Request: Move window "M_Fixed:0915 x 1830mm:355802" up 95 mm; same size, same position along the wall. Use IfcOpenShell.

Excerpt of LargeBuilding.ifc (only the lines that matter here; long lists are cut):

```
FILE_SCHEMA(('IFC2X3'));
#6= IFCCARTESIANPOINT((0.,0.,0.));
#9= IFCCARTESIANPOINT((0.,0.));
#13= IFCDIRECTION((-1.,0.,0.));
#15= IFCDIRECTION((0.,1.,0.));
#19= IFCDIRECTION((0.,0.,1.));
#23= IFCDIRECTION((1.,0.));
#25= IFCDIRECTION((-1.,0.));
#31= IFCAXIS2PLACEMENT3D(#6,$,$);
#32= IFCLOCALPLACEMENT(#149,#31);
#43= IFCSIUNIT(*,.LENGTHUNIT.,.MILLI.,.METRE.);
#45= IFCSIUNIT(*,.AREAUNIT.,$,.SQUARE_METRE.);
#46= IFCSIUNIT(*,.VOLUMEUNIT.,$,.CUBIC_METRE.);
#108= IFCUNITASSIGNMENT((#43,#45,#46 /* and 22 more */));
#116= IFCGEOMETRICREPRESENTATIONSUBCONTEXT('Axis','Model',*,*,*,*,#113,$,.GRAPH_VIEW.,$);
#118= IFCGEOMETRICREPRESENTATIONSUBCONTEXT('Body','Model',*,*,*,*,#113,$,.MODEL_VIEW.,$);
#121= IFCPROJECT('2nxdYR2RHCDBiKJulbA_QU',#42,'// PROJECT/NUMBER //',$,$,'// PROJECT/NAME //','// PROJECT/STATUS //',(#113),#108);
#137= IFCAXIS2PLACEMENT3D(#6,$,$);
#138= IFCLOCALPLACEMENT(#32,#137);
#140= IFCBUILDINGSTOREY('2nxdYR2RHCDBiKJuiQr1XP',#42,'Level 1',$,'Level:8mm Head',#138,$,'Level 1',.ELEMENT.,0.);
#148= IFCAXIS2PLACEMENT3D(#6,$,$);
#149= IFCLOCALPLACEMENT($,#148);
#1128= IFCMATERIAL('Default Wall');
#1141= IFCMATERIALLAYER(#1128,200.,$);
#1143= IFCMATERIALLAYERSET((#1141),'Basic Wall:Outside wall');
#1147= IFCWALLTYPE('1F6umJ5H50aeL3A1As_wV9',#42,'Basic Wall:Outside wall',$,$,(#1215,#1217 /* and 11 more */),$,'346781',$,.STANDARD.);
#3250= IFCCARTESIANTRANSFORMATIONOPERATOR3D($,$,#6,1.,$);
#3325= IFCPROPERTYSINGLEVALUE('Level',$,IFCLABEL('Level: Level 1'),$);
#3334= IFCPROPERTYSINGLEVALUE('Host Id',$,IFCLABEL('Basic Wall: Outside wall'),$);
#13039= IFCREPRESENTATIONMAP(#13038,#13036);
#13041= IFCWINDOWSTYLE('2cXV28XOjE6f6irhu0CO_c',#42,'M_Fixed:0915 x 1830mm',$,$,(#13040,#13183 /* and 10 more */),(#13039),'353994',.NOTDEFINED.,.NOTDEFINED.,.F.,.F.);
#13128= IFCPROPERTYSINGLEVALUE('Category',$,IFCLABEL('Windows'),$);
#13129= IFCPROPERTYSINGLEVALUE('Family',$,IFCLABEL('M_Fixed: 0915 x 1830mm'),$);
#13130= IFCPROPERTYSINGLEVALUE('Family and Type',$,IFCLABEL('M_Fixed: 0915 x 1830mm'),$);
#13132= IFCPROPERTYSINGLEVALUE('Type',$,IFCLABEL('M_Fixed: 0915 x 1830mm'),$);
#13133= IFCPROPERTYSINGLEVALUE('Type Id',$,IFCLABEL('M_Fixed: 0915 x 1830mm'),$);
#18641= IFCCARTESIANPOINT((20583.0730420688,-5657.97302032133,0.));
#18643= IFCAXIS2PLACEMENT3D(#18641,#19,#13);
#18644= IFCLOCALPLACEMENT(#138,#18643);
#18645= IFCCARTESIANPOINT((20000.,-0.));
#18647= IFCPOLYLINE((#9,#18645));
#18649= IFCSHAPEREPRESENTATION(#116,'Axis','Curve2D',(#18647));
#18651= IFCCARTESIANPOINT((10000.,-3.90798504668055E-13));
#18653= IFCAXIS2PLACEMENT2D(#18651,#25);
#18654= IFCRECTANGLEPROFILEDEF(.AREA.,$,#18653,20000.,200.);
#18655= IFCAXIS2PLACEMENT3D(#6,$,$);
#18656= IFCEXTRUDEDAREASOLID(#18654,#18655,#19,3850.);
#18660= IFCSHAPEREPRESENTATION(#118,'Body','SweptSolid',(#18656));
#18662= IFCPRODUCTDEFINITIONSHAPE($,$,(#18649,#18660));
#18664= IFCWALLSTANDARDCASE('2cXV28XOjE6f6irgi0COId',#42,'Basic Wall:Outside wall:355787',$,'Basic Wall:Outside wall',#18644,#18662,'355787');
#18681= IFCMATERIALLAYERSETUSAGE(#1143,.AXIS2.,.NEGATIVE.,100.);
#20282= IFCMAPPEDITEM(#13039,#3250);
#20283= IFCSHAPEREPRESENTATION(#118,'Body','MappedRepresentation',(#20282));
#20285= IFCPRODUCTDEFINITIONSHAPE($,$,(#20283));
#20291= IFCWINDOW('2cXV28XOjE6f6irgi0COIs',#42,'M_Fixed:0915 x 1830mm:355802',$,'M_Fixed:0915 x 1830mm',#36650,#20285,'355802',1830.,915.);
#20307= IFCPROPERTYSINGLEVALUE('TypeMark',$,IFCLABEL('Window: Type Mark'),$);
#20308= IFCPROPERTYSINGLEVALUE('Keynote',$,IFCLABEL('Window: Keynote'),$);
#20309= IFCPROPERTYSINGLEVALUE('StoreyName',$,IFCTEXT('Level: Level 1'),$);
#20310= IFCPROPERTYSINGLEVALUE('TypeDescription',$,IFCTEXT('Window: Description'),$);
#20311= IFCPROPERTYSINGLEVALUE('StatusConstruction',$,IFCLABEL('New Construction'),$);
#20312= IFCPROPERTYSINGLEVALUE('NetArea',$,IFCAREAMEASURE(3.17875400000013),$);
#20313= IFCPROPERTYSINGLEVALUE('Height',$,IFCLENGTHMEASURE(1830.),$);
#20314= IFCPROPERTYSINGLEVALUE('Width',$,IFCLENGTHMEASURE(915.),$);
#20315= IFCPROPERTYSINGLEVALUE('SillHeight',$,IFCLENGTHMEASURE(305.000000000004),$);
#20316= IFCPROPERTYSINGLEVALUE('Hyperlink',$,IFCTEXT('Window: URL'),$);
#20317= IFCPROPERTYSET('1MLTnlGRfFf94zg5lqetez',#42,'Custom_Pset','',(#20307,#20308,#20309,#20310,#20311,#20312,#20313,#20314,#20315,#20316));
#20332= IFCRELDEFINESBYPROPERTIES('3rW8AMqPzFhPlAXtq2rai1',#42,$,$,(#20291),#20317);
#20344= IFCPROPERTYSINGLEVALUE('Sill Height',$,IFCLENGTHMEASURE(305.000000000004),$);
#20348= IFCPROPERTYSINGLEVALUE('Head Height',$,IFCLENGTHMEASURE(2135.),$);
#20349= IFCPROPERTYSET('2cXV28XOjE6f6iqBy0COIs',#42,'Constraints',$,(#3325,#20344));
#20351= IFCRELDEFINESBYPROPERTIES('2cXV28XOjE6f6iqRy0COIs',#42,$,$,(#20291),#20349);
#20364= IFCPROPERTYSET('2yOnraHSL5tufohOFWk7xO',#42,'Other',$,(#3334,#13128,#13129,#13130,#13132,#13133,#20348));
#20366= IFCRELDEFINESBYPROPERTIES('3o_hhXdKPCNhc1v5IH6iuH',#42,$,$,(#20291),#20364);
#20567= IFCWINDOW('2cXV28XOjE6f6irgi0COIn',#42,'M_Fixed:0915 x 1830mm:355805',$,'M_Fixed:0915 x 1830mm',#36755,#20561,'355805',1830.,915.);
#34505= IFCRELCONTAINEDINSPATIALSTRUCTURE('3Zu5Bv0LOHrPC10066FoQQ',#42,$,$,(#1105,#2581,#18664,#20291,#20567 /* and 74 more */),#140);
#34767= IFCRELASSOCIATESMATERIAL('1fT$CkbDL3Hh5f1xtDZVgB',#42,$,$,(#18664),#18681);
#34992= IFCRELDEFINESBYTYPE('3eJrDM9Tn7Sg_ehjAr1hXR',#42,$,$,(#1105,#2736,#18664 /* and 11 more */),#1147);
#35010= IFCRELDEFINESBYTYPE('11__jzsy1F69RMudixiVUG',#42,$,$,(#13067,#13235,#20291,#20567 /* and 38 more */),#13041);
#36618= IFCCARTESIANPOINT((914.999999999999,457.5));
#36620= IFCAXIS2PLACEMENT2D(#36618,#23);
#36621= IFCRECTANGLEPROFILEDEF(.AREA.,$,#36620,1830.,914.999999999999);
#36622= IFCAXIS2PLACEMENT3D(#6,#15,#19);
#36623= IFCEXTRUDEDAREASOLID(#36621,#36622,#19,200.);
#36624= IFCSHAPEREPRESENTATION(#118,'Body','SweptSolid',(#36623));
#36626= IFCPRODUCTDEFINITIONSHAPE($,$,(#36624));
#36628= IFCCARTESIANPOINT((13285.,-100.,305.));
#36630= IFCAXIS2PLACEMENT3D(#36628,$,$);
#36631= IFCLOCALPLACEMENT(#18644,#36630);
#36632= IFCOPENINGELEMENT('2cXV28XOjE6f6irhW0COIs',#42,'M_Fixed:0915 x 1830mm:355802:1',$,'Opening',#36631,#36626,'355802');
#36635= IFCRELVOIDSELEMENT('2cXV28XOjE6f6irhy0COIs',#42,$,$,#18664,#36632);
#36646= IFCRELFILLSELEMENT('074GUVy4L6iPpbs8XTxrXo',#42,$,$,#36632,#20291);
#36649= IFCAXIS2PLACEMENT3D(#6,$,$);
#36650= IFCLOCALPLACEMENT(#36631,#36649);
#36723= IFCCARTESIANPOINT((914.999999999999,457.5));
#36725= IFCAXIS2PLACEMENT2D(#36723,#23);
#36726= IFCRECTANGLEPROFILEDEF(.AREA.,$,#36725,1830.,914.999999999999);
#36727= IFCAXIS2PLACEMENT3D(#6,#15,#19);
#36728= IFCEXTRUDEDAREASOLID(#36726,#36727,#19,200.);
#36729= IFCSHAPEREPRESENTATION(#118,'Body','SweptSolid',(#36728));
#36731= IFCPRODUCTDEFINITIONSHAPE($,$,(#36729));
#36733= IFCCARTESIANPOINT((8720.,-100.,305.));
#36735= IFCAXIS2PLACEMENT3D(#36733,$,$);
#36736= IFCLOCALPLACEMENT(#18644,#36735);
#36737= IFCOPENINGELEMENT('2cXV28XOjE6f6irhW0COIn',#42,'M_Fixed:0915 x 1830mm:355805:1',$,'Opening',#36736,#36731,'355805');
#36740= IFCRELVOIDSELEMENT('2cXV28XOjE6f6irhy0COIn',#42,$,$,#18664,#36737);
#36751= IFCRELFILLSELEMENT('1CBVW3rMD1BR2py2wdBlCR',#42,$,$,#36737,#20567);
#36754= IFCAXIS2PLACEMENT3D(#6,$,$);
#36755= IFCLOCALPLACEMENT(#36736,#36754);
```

```python
import numpy as np
import ifcopenshell
import ifcopenshell.api.geometry
import ifcopenshell.api.pset
import ifcopenshell.util.element
import ifcopenshell.util.placement
import ifcopenshell.util.unit

model = ifcopenshell.open("LargeBuilding.ifc")
unit_scale = ifcopenshell.util.unit.calculate_unit_scale(model)

window = model.by_id(20291)
opening = window.FillsVoids[0].RelatingOpeningElement
dz = 95.0

shift = np.array([0.0, 0.0, dz])
# The window is placed relative to its opening, so it follows when the opening moves.
matrix = ifcopenshell.util.placement.get_local_placement(opening.ObjectPlacement)
matrix[:3, 3] += shift
ifcopenshell.api.geometry.edit_object_placement(
    model, product=opening, matrix=matrix, is_si=False, should_transform_children=True
)

# Keep the stored heights in step.
pset = model.by_id(ifcopenshell.util.element.get_pset(window, "Custom_Pset", should_inherit=False)["id"])
ifcopenshell.api.pset.edit_pset(model, pset=pset, properties={
    "SillHeight": model.create_entity("IfcLengthMeasure", ifcopenshell.util.element.get_pset(window, "Constraints", "Sill Height") + dz),
})
pset = model.by_id(ifcopenshell.util.element.get_pset(window, "Constraints", should_inherit=False)["id"])
ifcopenshell.api.pset.edit_pset(model, pset=pset, properties={
    "Sill Height": model.create_entity("IfcLengthMeasure", ifcopenshell.util.element.get_pset(window, "Constraints", "Sill Height") + dz),
})
pset = model.by_id(ifcopenshell.util.element.get_pset(window, "Other", should_inherit=False)["id"])
ifcopenshell.api.pset.edit_pset(model, pset=pset, properties={
    "Head Height": model.create_entity("IfcLengthMeasure", ifcopenshell.util.element.get_pset(window, "Other", "Head Height") + dz),
})

print(f"moved by {dz * unit_scale:+.3f} m")

model.write("LargeBuilding_edited.ifc")
```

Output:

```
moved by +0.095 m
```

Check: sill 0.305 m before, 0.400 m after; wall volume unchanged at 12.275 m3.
